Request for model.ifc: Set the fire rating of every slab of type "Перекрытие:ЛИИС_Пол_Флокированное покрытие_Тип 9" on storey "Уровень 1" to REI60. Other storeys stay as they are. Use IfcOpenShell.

First a look at what the model holds.

```python
import ifcopenshell
import ifcopenshell.util.element

model = ifcopenshell.open("model.ifc")
print(model.schema)
storey = next(s for s in model.by_type("IfcBuildingStorey") if s.Name == "Уровень 1")
slabs = [e for e in ifcopenshell.util.element.get_decomposition(storey) if e.is_a("IfcSlab")]
seen = {}
for e in slabs:
    element_type = ifcopenshell.util.element.get_type(e)
    key = (element_type.Name if element_type != e and element_type else None, ifcopenshell.util.element.get_pset(e, "Pset_SlabCommon", "FireRating"))
    seen[key] = seen.get(key, 0) + 1
for (name, value), count in sorted(seen.items(), key=str):
    print(count, "x", name, "|", value)
```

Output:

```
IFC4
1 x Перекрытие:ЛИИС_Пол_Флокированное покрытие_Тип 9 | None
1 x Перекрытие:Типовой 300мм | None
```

```python
import ifcopenshell
import ifcopenshell.api.pset
import ifcopenshell.util.element

model = ifcopenshell.open("model.ifc")

storey = next(s for s in model.by_type("IfcBuildingStorey") if s.Name == "Уровень 1")
slabs = [e for e in ifcopenshell.util.element.get_decomposition(storey) if e.is_a("IfcSlab")]

count = 0
for e in slabs:
    element_type = ifcopenshell.util.element.get_type(e)
    if element_type in (None, e) or element_type.Name != "Перекрытие:ЛИИС_Пол_Флокированное покрытие_Тип 9":
        continue
    # add_pset returns the element's existing set when there is one.
    pset = ifcopenshell.api.pset.add_pset(model, product=e, name="Pset_SlabCommon")
    ifcopenshell.api.pset.edit_pset(model, pset=pset, properties={"FireRating": "REI60"})
    count += 1

print(count, "slabs updated")

model.write("model-out.ifc")
```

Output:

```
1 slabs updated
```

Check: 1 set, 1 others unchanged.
